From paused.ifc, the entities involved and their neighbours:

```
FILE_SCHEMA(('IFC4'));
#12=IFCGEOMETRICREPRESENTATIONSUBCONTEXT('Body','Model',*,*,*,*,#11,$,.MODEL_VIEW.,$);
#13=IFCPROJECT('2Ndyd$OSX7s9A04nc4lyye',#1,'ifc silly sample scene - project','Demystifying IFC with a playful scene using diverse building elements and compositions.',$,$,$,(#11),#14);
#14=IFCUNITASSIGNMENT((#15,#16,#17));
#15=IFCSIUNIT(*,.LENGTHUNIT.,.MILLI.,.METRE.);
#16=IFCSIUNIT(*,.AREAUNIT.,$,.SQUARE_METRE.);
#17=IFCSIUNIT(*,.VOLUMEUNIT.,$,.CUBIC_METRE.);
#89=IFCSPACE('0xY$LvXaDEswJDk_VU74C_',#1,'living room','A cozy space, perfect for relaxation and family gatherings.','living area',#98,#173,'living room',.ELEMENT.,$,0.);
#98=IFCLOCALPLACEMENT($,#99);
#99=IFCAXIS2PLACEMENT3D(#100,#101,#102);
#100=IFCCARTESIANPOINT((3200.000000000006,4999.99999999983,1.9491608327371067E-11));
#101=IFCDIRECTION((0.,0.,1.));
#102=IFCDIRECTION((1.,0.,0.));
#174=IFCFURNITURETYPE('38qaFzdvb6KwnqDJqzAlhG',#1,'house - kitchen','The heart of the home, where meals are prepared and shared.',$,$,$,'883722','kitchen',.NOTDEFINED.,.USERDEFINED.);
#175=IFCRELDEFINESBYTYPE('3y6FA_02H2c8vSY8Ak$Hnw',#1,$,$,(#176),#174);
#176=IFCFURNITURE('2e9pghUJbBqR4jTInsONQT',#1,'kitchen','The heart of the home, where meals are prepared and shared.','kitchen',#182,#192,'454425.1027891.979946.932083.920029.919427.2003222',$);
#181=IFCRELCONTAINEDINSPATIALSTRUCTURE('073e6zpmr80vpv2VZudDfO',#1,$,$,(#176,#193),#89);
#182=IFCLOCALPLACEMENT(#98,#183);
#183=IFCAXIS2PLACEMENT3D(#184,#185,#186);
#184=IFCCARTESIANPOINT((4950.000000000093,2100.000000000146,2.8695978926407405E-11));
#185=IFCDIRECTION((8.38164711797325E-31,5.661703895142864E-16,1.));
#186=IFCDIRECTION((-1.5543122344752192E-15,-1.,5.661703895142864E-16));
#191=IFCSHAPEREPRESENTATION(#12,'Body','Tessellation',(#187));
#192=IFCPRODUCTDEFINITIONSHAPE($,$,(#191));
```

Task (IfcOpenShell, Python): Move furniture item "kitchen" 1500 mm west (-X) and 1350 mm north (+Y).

```python
import ifcopenshell
import ifcopenshell.api.geometry
import ifcopenshell.util.placement

model = ifcopenshell.open("paused.ifc")

item = model.by_guid("2e9pghUJbBqR4jTInsONQT")
matrix = ifcopenshell.util.placement.get_local_placement(item.ObjectPlacement)
matrix[0, 3] -= 1500.0
matrix[1, 3] += 1350.0
ifcopenshell.api.geometry.edit_object_placement(model, product=item, matrix=matrix, is_si=False)

print(ifcopenshell.util.placement.get_local_placement(item.ObjectPlacement).round(3) + 0.0)

model.write("paused-out.ifc")
```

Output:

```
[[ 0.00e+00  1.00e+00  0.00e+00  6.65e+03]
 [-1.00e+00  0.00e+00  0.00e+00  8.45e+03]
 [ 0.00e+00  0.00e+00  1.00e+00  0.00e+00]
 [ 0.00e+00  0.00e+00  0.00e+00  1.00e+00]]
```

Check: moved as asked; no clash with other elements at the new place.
